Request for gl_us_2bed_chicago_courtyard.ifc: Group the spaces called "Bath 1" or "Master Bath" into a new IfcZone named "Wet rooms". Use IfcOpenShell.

First a look at what the model holds.

```python
import ifcopenshell

model = ifcopenshell.open("gl_us_2bed_chicago_courtyard.ifc")
print(model.schema)
seen = {}
for space in model.by_type("IfcSpace"):
    seen[space.LongName] = seen.get(space.LongName, 0) + 1
for name, count in sorted(seen.items(), key=str):
    print(count, "x", name)
print("zones:", [z.Name for z in model.by_type("IfcZone")][:20])
```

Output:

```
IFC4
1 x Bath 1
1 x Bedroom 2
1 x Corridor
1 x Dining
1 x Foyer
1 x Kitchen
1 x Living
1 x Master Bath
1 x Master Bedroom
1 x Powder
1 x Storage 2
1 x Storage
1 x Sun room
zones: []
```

```python
import ifcopenshell
import ifcopenshell.api.group
import ifcopenshell.api.root

model = ifcopenshell.open("gl_us_2bed_chicago_courtyard.ifc")

names = {"Bath 1", "Master Bath"}
spaces = [s for s in model.by_type("IfcSpace") if s.LongName in names]

zone = ifcopenshell.api.root.create_entity(model, ifc_class="IfcZone", name="Wet rooms")
ifcopenshell.api.group.assign_group(model, products=spaces, group=zone)
print(len(spaces), "spaces in", zone.Name)

model.write("gl_us_2bed_chicago_courtyard_v2.ifc")
```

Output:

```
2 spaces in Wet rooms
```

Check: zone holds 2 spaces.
